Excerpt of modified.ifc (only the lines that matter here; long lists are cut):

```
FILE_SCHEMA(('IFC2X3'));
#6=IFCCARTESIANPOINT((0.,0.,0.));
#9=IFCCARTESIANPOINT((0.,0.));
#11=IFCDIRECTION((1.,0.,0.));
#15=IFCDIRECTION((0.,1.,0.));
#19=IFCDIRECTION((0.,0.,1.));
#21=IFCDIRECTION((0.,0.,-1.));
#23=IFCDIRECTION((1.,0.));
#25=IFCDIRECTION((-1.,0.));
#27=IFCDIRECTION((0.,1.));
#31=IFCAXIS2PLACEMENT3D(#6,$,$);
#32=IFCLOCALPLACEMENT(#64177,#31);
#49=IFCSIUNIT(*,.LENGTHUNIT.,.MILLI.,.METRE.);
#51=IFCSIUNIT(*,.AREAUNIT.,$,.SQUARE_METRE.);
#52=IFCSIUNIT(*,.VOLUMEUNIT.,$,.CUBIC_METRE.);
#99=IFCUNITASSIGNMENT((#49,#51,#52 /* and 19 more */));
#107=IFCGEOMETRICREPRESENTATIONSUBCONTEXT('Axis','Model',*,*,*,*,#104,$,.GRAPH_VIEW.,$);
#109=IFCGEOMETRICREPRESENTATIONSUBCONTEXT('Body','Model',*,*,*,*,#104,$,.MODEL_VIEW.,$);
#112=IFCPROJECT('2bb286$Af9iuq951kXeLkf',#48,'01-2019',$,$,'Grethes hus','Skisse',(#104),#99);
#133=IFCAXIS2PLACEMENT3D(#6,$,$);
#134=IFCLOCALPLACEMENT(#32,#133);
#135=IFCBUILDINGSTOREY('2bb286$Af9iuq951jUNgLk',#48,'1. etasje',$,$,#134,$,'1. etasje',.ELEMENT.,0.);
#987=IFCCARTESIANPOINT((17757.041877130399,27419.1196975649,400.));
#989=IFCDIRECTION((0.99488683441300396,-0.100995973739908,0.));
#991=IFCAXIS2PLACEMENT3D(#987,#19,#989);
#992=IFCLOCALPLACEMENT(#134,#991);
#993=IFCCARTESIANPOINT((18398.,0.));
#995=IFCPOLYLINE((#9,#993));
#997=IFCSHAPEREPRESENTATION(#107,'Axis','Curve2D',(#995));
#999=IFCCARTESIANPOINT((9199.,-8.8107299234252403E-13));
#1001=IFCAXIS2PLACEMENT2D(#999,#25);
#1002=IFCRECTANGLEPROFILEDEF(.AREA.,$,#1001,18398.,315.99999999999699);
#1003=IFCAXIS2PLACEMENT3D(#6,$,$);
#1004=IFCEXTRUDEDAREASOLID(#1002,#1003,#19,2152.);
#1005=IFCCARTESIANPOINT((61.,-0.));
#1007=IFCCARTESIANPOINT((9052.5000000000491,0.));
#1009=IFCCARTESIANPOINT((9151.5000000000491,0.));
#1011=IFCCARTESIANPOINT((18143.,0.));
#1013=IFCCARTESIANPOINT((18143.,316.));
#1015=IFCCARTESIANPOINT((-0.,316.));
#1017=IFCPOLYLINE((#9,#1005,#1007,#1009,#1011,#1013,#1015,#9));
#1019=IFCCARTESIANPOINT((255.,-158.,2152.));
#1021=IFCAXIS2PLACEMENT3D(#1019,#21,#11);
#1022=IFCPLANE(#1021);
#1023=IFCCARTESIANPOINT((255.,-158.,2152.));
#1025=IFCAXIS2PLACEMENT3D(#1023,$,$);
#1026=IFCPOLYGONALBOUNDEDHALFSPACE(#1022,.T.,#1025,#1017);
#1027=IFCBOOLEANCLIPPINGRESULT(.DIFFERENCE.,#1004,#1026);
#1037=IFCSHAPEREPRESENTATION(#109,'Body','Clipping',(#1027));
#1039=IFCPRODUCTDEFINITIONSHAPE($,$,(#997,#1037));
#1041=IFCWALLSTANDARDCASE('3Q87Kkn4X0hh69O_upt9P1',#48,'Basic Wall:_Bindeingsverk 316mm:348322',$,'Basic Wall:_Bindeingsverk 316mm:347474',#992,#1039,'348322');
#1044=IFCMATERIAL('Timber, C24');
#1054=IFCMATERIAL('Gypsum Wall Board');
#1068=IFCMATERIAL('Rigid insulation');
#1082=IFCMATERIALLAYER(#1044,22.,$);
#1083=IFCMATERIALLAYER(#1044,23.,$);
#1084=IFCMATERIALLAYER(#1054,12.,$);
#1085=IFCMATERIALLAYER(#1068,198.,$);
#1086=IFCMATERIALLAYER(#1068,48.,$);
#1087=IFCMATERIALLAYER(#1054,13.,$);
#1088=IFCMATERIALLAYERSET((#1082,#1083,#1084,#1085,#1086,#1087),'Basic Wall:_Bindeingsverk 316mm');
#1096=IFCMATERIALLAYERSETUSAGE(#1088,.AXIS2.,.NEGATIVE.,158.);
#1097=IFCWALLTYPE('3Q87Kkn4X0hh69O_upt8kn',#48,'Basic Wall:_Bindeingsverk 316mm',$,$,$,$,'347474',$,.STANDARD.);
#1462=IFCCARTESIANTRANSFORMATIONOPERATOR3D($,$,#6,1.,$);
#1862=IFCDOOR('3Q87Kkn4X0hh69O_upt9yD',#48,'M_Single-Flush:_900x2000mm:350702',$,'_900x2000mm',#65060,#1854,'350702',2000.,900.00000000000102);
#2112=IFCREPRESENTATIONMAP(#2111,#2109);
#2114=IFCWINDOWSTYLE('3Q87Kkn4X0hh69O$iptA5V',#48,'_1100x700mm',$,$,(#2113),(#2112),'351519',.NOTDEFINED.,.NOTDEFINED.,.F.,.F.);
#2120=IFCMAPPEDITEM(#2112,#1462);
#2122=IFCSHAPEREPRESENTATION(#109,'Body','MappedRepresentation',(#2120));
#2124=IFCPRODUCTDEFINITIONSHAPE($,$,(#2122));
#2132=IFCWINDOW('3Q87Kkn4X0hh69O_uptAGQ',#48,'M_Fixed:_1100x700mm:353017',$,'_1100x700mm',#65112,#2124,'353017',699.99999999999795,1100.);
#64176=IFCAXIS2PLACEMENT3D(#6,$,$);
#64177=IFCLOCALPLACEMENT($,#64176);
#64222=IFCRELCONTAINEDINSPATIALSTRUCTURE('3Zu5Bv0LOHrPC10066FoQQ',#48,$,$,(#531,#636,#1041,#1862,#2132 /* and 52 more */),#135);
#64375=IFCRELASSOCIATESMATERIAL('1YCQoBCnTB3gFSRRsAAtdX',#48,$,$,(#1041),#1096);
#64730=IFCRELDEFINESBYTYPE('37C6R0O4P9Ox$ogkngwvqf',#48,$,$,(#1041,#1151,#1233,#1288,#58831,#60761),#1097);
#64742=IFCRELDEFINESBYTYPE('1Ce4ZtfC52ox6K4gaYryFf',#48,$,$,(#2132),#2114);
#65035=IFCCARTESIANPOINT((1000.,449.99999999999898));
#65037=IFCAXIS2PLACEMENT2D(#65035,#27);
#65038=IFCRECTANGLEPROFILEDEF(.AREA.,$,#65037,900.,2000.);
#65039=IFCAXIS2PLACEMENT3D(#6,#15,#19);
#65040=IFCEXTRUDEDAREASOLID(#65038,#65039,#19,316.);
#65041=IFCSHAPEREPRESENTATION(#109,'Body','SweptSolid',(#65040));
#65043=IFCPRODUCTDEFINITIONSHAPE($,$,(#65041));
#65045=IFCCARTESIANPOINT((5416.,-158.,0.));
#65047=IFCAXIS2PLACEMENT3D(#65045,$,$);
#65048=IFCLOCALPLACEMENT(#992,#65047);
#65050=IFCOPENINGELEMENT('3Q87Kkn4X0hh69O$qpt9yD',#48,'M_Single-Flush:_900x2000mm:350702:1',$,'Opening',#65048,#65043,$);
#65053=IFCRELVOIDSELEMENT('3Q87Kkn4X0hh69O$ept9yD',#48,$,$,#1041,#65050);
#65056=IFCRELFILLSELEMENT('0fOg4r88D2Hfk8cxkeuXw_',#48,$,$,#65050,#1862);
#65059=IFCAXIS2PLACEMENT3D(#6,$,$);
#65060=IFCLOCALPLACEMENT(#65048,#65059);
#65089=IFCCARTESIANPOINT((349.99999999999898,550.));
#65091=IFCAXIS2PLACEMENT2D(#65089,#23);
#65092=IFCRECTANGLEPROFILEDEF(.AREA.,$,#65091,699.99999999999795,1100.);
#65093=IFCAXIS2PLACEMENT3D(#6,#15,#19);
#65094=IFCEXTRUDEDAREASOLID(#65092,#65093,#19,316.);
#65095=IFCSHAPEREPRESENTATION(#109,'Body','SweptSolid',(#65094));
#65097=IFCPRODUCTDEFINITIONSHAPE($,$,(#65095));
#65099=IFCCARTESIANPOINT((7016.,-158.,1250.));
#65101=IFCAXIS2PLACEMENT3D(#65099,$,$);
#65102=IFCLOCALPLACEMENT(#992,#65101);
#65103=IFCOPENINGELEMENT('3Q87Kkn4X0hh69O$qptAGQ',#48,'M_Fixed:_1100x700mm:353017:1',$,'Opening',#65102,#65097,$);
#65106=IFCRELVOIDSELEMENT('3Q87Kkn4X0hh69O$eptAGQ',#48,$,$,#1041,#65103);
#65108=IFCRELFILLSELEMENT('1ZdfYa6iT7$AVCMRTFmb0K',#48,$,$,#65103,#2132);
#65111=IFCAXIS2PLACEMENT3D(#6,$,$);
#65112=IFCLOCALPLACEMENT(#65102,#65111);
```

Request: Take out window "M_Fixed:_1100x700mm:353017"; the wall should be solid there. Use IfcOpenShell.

```python
import ifcopenshell
import ifcopenshell.api.feature
import ifcopenshell.api.root
import ifcopenshell.geom
import ifcopenshell.util.shape

model = ifcopenshell.open("modified.ifc")
settings = ifcopenshell.geom.settings()


def volume(element):
    """Net volume in cubic metres, openings subtracted."""
    shape = ifcopenshell.geom.create_shape(settings, element)
    return ifcopenshell.util.shape.get_volume(shape.geometry)


window = model.by_id(2132)
opening = window.FillsVoids[0].RelatingOpeningElement
wall = opening.VoidsElements[0].RelatingBuildingElement
before = volume(wall)

ifcopenshell.api.root.remove_product(model, product=window)
ifcopenshell.api.feature.remove_feature(model, feature=opening)

after = volume(wall)

print(f"wall volume {before:.3f} -> {after:.3f} m3")

model.write("modified-out.ifc")
```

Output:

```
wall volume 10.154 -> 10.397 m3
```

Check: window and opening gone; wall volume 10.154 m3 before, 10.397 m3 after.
